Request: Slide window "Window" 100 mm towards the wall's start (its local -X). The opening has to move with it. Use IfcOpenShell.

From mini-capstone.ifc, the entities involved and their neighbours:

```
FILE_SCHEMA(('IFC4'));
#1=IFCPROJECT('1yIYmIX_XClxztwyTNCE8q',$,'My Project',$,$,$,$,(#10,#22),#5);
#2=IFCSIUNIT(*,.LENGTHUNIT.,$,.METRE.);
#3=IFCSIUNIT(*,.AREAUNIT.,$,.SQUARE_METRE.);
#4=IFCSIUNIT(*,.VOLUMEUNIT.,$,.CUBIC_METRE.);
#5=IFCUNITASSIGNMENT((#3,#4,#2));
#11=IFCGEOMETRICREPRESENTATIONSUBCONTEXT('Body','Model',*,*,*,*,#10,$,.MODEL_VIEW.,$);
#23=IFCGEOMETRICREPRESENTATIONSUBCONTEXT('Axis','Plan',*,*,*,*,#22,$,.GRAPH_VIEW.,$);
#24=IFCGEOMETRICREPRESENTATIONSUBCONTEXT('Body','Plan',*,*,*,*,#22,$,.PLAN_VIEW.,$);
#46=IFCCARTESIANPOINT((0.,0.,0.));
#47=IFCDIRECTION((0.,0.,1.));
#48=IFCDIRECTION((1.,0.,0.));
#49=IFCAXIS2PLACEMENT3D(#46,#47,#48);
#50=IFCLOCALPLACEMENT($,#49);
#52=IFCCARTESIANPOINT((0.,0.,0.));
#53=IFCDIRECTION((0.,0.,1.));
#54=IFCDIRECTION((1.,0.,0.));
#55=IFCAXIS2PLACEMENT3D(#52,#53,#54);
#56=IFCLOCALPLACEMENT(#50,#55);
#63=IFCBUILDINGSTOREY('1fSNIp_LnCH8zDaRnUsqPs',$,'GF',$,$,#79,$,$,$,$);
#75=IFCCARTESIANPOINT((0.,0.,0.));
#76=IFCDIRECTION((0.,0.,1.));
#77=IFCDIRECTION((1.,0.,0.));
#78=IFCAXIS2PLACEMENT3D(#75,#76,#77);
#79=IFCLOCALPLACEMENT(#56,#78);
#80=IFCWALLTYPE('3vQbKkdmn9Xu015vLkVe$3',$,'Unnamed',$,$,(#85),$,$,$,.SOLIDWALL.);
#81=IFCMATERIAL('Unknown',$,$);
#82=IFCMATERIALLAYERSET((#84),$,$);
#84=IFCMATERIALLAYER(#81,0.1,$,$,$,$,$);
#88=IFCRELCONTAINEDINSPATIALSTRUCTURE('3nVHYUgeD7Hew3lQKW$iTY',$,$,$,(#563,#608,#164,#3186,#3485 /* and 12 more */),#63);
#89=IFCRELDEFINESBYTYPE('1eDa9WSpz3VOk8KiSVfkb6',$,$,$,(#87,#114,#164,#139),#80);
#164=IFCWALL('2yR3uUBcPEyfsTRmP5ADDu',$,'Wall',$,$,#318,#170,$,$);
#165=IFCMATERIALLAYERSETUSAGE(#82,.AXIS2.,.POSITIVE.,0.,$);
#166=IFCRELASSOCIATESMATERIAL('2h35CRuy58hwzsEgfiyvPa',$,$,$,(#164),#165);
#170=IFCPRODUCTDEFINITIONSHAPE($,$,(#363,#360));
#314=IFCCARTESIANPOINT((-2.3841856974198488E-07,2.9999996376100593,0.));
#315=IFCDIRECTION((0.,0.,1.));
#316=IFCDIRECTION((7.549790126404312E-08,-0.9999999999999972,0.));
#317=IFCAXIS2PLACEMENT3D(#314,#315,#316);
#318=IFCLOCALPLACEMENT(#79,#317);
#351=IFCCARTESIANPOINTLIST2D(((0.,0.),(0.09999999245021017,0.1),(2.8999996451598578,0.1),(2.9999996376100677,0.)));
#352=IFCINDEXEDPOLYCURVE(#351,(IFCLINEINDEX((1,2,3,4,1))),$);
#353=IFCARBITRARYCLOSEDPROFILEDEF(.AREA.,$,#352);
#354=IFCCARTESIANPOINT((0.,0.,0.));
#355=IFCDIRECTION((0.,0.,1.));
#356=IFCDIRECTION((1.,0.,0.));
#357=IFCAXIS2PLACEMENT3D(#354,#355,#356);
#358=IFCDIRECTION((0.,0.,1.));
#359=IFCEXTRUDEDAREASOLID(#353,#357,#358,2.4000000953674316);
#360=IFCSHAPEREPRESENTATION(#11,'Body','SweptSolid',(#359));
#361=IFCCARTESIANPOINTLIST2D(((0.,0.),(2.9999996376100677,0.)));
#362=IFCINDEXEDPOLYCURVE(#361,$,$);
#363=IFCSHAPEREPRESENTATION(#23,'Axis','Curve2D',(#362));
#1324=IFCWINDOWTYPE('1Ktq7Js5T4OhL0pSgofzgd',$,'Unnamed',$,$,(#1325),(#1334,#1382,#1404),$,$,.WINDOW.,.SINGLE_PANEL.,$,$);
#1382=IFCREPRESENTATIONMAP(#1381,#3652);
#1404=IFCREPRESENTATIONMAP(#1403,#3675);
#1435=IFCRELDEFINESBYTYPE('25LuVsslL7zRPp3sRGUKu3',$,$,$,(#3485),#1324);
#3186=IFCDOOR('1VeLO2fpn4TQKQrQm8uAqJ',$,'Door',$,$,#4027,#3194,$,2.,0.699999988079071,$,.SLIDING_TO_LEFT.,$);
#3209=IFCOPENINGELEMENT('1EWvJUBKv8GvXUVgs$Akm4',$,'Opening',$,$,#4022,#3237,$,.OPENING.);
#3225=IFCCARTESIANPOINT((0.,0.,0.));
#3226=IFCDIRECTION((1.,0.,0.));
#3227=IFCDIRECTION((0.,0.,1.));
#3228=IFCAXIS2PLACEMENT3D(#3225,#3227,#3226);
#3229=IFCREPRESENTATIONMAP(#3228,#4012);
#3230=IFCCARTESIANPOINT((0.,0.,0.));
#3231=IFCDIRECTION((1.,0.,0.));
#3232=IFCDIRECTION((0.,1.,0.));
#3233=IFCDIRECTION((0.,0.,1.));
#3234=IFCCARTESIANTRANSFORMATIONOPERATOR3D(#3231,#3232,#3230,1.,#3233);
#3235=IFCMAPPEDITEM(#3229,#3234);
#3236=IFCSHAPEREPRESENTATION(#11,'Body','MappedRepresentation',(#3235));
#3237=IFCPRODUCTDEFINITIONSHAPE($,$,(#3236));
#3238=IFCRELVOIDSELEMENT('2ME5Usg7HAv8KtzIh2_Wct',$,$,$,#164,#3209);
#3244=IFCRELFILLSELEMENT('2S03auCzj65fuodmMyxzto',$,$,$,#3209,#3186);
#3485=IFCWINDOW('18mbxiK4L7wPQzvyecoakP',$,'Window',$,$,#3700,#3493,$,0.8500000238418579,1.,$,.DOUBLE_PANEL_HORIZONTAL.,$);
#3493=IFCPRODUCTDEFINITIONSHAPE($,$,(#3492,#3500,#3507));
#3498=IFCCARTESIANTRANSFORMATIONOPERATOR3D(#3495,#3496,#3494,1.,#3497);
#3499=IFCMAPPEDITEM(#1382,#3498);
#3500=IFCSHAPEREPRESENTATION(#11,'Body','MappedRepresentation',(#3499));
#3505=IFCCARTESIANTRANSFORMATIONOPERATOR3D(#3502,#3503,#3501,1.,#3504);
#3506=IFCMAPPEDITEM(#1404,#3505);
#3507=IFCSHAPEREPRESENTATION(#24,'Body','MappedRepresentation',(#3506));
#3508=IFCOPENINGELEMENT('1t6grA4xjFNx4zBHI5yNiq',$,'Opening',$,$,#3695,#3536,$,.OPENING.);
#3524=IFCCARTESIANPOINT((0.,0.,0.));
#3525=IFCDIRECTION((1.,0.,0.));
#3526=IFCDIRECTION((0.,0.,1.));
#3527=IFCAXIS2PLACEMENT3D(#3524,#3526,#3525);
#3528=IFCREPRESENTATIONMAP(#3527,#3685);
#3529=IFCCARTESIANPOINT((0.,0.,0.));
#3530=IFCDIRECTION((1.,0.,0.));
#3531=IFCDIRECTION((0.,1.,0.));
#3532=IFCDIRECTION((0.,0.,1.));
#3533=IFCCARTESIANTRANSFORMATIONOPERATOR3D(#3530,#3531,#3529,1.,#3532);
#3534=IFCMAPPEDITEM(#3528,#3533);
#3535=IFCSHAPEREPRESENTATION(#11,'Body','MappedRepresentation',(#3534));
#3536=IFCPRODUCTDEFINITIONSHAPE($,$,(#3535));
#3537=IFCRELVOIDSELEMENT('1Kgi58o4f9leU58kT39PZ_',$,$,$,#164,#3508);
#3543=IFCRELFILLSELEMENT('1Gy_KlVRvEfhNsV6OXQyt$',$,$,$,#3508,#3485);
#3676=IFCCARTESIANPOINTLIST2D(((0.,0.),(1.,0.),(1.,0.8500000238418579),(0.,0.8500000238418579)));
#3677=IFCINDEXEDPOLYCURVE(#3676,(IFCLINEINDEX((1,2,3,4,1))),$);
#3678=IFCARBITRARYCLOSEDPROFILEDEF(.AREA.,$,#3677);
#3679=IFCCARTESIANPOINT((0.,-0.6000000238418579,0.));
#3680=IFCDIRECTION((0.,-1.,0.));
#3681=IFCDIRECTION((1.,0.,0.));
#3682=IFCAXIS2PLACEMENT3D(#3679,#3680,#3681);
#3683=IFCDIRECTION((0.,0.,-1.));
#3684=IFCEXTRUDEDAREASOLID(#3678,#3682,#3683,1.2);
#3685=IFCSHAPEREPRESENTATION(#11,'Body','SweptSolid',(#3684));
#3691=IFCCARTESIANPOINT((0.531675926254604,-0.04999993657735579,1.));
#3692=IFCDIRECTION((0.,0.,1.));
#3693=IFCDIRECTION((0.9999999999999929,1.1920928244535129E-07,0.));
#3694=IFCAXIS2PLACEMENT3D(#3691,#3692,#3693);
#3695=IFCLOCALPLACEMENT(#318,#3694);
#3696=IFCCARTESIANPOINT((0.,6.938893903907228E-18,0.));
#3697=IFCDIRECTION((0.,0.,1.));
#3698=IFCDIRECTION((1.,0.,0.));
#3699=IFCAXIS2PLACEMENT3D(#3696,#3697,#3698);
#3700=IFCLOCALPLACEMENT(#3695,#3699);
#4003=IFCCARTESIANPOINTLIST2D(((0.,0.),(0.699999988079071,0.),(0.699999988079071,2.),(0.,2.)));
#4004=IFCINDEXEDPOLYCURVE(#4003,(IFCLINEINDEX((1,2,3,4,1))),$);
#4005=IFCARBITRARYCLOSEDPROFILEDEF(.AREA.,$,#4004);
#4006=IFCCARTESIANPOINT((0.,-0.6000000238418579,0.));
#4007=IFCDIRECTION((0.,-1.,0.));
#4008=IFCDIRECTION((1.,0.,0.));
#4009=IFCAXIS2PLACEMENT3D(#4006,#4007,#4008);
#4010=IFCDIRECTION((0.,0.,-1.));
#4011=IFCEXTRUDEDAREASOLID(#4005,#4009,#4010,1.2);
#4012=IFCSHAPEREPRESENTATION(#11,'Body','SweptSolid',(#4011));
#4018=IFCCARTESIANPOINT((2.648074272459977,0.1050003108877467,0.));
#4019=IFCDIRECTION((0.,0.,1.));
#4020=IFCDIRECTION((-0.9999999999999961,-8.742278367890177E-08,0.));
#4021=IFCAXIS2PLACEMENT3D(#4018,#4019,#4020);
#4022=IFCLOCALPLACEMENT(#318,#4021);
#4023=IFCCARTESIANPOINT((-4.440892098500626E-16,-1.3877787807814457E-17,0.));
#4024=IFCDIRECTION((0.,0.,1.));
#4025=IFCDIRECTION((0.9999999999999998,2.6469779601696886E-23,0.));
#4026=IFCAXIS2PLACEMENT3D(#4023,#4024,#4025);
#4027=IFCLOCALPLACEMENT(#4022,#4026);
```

```python
import ifcopenshell
import ifcopenshell.api.geometry
import ifcopenshell.util.placement

model = ifcopenshell.open("mini-capstone.ifc")

window = model.by_guid("18mbxiK4L7wPQzvyecoakP")
opening = window.FillsVoids[0].RelatingOpeningElement
wall = opening.VoidsElements[0].RelatingBuildingElement

wall_matrix = ifcopenshell.util.placement.get_local_placement(wall.ObjectPlacement)
shift = wall_matrix[:3, 0] * -0.1
before = ifcopenshell.util.placement.get_local_placement(window.ObjectPlacement)[:3, 3].copy()

# The window is placed relative to its opening, so it follows when the opening moves.
matrix = ifcopenshell.util.placement.get_local_placement(opening.ObjectPlacement)
matrix[:3, 3] += shift
ifcopenshell.api.geometry.edit_object_placement(
    model, product=opening, matrix=matrix, is_si=False, should_transform_children=True
)

after = ifcopenshell.util.placement.get_local_placement(window.ObjectPlacement)[:3, 3]
print("window moved by", (after - before).round(3) + 0.0)

model.write("mini-capstone_rev.ifc")
```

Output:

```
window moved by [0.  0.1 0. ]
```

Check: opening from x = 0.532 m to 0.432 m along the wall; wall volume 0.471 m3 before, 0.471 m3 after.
